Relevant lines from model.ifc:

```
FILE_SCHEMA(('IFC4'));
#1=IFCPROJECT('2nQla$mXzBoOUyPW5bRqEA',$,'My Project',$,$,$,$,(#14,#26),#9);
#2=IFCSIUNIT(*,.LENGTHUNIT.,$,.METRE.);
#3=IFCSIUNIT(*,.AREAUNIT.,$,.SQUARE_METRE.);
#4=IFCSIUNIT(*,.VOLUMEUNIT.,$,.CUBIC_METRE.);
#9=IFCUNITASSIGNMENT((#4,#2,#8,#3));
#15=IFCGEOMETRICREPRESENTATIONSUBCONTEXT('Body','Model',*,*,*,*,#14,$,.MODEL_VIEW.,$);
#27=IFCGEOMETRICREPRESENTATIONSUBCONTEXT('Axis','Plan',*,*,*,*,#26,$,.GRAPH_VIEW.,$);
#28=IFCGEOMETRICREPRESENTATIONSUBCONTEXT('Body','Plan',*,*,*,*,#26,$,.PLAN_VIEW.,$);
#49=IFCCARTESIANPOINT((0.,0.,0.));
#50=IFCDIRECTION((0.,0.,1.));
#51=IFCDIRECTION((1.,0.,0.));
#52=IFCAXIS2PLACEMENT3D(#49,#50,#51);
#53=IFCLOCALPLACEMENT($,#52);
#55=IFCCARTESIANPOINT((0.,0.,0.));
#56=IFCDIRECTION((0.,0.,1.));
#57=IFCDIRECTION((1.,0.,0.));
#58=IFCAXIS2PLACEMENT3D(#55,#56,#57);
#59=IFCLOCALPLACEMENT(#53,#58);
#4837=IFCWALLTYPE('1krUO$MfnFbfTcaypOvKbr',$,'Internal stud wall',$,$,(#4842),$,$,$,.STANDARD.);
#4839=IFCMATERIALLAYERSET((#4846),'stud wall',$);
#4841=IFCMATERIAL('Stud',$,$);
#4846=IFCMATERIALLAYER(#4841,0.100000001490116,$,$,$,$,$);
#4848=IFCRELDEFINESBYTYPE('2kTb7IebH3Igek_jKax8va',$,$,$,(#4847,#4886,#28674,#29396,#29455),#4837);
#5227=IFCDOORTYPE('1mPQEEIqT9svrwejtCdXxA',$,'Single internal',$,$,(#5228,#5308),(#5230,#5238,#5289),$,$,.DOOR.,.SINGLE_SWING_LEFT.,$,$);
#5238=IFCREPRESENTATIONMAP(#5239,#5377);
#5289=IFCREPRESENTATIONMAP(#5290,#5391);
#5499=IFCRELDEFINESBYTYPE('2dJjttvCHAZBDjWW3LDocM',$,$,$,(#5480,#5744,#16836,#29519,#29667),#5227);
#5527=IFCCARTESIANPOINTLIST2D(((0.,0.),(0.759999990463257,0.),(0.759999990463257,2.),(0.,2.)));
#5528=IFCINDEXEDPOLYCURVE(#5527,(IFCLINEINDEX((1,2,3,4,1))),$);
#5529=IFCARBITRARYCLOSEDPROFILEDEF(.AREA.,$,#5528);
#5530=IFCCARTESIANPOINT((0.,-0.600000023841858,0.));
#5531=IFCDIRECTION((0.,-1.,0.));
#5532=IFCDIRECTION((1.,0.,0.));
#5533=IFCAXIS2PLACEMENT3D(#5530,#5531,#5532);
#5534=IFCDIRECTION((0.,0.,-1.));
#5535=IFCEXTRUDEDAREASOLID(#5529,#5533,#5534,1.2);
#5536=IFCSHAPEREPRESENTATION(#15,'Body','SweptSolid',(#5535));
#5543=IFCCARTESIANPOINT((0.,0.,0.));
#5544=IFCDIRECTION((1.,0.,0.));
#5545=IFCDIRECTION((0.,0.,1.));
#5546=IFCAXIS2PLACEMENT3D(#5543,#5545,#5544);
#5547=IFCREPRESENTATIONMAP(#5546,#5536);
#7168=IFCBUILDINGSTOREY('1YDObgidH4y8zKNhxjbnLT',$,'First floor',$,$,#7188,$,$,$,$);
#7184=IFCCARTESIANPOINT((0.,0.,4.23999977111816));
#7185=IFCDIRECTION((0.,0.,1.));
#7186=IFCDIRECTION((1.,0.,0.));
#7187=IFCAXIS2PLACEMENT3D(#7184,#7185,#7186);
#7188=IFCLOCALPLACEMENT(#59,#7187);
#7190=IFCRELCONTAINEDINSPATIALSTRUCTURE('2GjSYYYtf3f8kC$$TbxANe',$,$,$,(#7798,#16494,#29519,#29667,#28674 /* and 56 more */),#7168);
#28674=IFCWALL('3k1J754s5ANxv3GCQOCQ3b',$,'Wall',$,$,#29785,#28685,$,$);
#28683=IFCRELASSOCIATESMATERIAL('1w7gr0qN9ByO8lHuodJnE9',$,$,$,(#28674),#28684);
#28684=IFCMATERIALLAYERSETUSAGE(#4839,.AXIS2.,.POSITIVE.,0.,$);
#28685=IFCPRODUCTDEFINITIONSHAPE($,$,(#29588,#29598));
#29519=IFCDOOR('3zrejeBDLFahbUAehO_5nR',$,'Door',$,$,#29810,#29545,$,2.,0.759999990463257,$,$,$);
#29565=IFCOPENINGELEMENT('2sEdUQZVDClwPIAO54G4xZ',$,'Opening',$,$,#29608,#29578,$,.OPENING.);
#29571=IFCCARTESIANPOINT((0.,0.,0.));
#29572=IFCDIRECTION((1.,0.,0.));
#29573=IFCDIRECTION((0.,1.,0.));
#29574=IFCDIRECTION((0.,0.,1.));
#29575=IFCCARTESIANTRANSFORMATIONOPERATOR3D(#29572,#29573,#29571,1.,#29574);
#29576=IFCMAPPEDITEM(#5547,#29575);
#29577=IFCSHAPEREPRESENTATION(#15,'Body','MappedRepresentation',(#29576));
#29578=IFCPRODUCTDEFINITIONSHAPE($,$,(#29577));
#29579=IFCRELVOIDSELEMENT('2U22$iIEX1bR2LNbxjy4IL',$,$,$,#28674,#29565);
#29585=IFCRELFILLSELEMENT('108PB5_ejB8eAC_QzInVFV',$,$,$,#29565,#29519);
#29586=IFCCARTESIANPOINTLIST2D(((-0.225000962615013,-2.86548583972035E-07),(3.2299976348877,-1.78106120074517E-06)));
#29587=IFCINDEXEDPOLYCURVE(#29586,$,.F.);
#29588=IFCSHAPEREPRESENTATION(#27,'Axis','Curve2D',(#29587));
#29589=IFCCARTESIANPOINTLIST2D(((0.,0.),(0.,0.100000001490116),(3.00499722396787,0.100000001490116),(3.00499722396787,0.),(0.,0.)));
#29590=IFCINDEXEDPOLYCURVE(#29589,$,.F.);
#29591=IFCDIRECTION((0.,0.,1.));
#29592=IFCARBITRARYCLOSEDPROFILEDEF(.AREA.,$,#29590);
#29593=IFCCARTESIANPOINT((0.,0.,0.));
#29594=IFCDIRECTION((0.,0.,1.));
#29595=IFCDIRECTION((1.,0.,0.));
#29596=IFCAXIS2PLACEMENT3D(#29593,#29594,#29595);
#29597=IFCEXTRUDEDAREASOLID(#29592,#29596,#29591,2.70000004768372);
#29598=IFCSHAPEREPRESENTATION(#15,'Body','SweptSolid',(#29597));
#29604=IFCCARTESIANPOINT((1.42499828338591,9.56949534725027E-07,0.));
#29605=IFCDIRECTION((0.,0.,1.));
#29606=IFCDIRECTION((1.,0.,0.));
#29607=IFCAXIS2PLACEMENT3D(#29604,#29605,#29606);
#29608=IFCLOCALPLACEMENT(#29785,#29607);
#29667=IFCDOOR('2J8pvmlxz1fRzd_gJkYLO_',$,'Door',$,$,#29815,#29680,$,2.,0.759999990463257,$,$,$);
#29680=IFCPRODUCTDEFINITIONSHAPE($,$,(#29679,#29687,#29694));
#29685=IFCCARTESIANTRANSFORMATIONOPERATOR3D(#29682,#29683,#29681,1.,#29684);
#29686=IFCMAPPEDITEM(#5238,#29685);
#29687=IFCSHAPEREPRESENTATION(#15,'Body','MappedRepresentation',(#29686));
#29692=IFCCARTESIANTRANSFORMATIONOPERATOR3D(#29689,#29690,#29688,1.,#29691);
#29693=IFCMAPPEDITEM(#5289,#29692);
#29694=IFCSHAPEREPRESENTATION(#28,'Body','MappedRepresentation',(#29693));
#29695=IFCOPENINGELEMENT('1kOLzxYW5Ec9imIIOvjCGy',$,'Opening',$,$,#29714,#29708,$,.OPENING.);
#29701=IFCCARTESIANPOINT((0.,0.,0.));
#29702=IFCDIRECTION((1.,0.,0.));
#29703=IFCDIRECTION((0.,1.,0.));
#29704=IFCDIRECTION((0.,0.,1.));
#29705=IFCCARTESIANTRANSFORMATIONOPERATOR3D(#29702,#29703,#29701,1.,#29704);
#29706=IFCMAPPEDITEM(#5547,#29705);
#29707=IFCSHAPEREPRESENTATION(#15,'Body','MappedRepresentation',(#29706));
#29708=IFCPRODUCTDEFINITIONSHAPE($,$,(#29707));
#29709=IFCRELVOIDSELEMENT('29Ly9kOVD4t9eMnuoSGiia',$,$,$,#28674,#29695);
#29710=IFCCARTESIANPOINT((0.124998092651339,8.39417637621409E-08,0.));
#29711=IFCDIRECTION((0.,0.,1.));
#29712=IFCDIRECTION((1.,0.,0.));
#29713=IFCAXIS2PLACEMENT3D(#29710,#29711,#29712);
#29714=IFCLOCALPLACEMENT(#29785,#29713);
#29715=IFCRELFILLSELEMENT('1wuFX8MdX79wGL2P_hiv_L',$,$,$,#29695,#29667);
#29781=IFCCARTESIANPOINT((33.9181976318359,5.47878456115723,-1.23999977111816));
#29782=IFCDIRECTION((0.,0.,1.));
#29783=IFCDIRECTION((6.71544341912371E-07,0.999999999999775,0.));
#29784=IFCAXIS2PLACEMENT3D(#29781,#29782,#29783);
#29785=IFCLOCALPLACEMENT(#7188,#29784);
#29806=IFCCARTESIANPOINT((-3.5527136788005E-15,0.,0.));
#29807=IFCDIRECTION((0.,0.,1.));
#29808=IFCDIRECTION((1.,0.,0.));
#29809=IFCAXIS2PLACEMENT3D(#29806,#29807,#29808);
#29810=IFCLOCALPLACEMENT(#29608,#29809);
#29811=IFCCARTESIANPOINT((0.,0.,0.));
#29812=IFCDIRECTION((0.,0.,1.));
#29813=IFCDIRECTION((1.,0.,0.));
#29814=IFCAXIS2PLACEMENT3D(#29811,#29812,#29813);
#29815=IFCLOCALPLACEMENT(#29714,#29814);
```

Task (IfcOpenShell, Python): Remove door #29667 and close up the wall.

```python
import ifcopenshell
import ifcopenshell.api.feature
import ifcopenshell.api.root
import ifcopenshell.geom
import ifcopenshell.util.shape

model = ifcopenshell.open("model.ifc")
settings = ifcopenshell.geom.settings()


def volume(element):
    """Net volume in cubic metres, openings subtracted."""
    shape = ifcopenshell.geom.create_shape(settings, element)
    return ifcopenshell.util.shape.get_volume(shape.geometry)


door = model.by_guid("2J8pvmlxz1fRzd_gJkYLO_")
opening = door.FillsVoids[0].RelatingOpeningElement
wall = opening.VoidsElements[0].RelatingBuildingElement
before = volume(wall)

ifcopenshell.api.root.remove_product(model, product=door)
ifcopenshell.api.feature.remove_feature(model, feature=opening)

after = volume(wall)

print(f"wall volume {before:.3f} -> {after:.3f} m3")

model.write("model_v2.ifc")
```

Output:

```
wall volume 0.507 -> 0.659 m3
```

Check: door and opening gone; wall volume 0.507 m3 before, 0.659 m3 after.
